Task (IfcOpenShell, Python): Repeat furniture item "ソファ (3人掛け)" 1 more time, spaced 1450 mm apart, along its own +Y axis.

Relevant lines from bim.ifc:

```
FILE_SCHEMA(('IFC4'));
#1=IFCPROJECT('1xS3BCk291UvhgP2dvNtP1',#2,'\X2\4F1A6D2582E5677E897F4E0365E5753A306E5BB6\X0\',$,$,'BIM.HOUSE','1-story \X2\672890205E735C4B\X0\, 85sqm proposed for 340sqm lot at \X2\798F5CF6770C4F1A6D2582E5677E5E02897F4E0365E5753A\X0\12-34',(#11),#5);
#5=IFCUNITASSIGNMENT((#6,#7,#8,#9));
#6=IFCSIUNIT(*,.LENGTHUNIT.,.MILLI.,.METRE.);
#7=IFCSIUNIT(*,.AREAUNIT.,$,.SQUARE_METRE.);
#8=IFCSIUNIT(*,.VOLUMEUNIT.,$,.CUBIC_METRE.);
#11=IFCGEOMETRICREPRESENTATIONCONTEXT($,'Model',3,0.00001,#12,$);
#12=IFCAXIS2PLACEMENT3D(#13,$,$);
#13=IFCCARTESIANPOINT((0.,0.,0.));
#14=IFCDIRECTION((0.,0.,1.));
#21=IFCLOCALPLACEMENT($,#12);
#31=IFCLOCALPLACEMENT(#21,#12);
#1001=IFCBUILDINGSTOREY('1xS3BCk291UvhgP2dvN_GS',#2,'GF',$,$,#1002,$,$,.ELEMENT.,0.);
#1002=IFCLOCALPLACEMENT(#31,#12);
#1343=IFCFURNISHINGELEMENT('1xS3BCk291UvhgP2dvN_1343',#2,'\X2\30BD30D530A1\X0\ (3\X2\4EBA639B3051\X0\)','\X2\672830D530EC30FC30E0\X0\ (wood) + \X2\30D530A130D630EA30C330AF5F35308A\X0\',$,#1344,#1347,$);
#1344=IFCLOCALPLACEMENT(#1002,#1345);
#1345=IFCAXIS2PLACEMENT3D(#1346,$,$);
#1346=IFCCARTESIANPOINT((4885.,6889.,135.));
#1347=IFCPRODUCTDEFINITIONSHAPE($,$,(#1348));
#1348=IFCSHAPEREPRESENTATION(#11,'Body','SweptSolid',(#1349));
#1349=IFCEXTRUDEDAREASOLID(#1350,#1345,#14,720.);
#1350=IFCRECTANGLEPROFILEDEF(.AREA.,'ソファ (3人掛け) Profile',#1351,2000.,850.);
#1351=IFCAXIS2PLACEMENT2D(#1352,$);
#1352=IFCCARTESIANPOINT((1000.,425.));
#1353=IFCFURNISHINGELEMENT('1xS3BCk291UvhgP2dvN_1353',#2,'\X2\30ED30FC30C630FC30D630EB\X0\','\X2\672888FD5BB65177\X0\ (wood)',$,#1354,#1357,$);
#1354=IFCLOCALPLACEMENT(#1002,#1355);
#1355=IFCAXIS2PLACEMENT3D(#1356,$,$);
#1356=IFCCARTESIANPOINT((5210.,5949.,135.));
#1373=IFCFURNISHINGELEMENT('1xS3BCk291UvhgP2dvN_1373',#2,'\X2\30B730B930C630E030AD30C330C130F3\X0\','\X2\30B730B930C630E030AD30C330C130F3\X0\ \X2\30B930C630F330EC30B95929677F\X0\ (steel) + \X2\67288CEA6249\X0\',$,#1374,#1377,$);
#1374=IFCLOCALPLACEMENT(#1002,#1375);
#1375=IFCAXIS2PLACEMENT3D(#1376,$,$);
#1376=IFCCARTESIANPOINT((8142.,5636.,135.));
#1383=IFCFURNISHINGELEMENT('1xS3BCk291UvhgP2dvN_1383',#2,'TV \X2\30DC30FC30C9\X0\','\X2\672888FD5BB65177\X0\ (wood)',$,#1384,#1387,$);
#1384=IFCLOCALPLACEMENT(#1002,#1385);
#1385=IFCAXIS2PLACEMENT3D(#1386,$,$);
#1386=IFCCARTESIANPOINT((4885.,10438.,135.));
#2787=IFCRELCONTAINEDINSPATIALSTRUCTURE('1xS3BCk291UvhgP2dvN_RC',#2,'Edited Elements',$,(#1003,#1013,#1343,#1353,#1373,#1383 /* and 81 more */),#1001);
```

```python
import ifcopenshell
import ifcopenshell.api.geometry
import ifcopenshell.api.root
import ifcopenshell.util.element
import ifcopenshell.util.placement
import ifcopenshell.util.unit

model = ifcopenshell.open("bim.ifc")
unit_scale = ifcopenshell.util.unit.calculate_unit_scale(model)


def reuse_history(source, copy):
    """copy_class also copies each property set's owner history, people and application; keep the originals."""
    for rel in copy.IsDefinedBy:
        if rel.is_a("IfcRelDefinesByProperties") and (history := rel.RelatingPropertyDefinition.OwnerHistory):
            rel.RelatingPropertyDefinition.OwnerHistory = source.OwnerHistory
            ifcopenshell.util.element.remove_deep2(model, history)


source = model.by_guid("1xS3BCk291UvhgP2dvN_1343")
base = ifcopenshell.util.placement.get_local_placement(source.ObjectPlacement)
step = base[:3, 1] * 1.45 / unit_scale

for i in range(1, 2):
    copy = ifcopenshell.api.root.copy_class(model, product=source)
    copy.Representation = ifcopenshell.util.element.copy_deep(
        model, source.Representation, exclude=["IfcGeometricRepresentationContext", "IfcRepresentationMap"]
    )
    reuse_history(source, copy)
    matrix = base.copy()
    matrix[:3, 3] += i * step
    print("added at", matrix[:3, 3].round(3) + 0.0)
    ifcopenshell.api.geometry.edit_object_placement(model, product=copy, matrix=matrix, is_si=False)

model.write("bim_v2.ifc")
```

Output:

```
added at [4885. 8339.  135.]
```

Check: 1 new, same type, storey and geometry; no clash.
